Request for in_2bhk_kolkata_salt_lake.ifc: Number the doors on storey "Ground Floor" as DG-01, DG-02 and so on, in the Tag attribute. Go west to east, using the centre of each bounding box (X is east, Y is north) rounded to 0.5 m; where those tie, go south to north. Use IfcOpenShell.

First a look at what the model holds.

```python
import ifcopenshell
import ifcopenshell.util.element
import ifcopenshell.util.placement

model = ifcopenshell.open("in_2bhk_kolkata_salt_lake.ifc")
print(model.schema)
storey = next(s for s in model.by_type("IfcBuildingStorey") if s.Name == "Ground Floor")
doors = [e for e in ifcopenshell.util.element.get_decomposition(storey) if e.is_a("IfcDoor")]
for e in sorted(doors, key=lambda e: e.id()):
    origin = ifcopenshell.util.placement.get_local_placement(e.ObjectPlacement)[:3, 3]
    print(e.id(), e.Tag, e.Name, origin.round(2) + 0.0, sep=" | ")
```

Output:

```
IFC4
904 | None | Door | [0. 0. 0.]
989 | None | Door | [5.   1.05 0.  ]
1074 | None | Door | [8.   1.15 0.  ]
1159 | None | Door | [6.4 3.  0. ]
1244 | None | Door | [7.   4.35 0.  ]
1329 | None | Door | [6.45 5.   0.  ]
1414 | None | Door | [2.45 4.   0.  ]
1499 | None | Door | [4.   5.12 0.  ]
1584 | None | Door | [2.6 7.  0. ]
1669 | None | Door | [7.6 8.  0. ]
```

```python
import ifcopenshell
import ifcopenshell.geom
import ifcopenshell.util.element
import ifcopenshell.util.shape

model = ifcopenshell.open("in_2bhk_kolkata_salt_lake.ifc")
settings = ifcopenshell.geom.settings()
settings.set("use-world-coords", True)


def centre(element):
    shape = ifcopenshell.geom.create_shape(settings, element)
    return ifcopenshell.util.shape.get_bbox_centroid(shape.geometry)


storey = next(s for s in model.by_type("IfcBuildingStorey") if s.Name == "Ground Floor")
doors = [e for e in ifcopenshell.util.element.get_decomposition(storey) if e.is_a("IfcDoor")]

# Insertion points can sit at a corner or the storey origin, so sort by the geometry (in metres).
centres = {e: centre(e) for e in doors}
doors.sort(key=lambda e: (round(centres[e][0] / 0.5), centres[e][1]))

for i, e in enumerate(doors, start=1):
    number = f"DG-{i:02d}"
    e.Tag = number
    print(e.id(), number)

model.write("in_2bhk_kolkata_salt_lake_v2.ifc")
```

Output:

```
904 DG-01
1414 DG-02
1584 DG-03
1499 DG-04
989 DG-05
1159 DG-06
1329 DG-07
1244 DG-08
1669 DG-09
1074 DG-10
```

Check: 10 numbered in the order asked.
